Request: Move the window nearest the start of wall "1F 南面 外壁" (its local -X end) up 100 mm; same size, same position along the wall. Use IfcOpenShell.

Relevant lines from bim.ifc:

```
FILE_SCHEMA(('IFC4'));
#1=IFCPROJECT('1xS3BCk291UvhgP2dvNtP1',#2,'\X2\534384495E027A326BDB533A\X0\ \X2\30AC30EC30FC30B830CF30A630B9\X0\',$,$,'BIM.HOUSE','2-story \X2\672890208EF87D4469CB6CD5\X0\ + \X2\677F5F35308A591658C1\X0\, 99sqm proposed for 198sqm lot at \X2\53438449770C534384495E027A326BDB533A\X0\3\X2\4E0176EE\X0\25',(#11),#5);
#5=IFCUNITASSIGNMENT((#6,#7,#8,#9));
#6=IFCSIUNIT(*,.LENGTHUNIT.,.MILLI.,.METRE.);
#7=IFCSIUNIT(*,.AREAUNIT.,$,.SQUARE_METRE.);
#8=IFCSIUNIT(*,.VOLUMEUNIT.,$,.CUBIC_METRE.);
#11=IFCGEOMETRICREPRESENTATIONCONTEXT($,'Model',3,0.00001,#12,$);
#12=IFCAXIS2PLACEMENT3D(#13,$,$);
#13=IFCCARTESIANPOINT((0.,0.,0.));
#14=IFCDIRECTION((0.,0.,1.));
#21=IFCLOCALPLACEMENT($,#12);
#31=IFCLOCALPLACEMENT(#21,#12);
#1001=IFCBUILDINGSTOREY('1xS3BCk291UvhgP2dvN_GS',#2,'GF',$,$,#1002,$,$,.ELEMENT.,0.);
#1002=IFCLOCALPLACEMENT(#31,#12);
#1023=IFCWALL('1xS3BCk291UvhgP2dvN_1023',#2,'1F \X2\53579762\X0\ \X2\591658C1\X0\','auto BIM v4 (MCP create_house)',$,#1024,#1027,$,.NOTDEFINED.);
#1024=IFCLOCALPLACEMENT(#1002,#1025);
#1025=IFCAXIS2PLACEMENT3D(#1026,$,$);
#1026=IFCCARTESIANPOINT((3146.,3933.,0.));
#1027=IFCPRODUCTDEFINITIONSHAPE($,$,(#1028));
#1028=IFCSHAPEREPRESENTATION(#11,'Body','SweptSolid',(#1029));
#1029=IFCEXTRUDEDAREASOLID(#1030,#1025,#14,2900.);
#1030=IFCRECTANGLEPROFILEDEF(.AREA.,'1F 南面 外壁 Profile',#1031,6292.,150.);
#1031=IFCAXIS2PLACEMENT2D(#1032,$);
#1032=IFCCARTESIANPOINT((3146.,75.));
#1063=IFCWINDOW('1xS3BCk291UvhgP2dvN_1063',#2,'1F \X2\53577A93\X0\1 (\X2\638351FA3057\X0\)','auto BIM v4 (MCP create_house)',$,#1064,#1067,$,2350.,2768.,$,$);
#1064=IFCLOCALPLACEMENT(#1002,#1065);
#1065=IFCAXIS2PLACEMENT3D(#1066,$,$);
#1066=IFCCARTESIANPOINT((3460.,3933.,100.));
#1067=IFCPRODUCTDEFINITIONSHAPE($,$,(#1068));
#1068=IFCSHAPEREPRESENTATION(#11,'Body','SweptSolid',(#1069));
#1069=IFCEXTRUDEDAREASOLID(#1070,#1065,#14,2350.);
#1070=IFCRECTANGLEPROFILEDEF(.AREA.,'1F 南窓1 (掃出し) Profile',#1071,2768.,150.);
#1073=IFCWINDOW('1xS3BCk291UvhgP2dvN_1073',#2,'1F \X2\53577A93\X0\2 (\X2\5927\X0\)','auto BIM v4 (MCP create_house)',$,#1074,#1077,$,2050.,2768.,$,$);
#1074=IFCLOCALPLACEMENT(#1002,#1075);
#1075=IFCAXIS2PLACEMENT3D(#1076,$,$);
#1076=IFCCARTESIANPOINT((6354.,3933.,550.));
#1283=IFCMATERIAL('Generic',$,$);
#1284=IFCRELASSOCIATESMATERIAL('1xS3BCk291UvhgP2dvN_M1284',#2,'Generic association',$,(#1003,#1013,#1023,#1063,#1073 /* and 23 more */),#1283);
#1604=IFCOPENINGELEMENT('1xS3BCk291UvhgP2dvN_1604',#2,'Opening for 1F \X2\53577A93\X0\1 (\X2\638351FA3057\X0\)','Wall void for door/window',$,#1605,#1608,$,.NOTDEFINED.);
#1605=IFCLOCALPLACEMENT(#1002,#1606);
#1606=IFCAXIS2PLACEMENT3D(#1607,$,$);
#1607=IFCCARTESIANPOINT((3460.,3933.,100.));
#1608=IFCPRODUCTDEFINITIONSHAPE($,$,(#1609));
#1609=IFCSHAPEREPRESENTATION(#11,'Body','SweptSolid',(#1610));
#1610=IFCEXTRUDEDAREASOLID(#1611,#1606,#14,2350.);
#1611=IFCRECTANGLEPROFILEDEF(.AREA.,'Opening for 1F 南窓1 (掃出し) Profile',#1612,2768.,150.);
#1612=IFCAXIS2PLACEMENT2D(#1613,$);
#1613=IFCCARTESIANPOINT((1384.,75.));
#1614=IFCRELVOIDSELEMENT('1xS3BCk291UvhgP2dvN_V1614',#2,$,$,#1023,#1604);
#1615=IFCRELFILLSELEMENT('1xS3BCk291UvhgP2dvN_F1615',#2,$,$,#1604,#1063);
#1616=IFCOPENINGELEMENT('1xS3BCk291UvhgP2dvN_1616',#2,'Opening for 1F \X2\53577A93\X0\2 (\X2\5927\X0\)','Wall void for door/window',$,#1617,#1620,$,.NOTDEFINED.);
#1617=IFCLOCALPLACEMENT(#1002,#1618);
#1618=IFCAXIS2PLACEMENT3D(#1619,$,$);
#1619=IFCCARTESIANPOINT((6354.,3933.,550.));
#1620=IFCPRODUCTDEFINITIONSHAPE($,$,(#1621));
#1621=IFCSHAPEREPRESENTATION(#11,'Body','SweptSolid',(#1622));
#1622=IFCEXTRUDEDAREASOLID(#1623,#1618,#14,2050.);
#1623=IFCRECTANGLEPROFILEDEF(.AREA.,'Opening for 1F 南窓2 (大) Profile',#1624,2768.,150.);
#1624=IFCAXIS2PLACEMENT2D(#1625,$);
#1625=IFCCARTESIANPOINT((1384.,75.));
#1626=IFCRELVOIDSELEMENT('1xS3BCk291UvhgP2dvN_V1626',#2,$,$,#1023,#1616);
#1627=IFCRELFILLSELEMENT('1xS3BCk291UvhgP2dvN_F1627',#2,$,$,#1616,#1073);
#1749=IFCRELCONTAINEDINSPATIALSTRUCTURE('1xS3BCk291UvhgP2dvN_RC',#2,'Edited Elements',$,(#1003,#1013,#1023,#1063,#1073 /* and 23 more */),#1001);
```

```python
import numpy as np
import ifcopenshell
import ifcopenshell.api.geometry
import ifcopenshell.util.placement
import ifcopenshell.util.unit

model = ifcopenshell.open("bim.ifc")
unit_scale = ifcopenshell.util.unit.calculate_unit_scale(model)

window = model.by_guid("1xS3BCk291UvhgP2dvN_1063")
opening = window.FillsVoids[0].RelatingOpeningElement
dz = 0.1 / unit_scale

shift = np.array([0.0, 0.0, dz])
# The window is not placed relative to its opening, so move both.
for product in (opening, window):
    matrix = ifcopenshell.util.placement.get_local_placement(product.ObjectPlacement)
    matrix[:3, 3] += shift
    ifcopenshell.api.geometry.edit_object_placement(model, product=product, matrix=matrix, is_si=False)

print(f"moved by {dz * unit_scale:+.3f} m")

model.write("bim_rev.ifc")
```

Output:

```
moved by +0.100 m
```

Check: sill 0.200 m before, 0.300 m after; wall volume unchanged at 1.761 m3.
